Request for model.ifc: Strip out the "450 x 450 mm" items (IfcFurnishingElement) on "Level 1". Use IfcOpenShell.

First a look at what the model holds.

```python
import ifcopenshell
import ifcopenshell.util.element

model = ifcopenshell.open("model.ifc")
print(model.schema)
storey = next(s for s in model.by_type("IfcBuildingStorey") if s.Name == "Level 1")
furniture = [e for e in ifcopenshell.util.element.get_decomposition(storey) if e.is_a("IfcFurnishingElement")]
seen = {}
for e in furniture:
    element_type = ifcopenshell.util.element.get_type(e)
    name = element_type.Name if element_type not in (None, e) else None
    seen[name] = seen.get(name, 0) + 1
for name, count in sorted(seen.items(), key=str):
    print(count, "x", name)
```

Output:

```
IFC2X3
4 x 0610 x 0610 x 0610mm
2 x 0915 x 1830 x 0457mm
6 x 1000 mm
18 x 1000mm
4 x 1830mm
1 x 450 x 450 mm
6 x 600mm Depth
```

```python
import ifcopenshell
import ifcopenshell.api.root
import ifcopenshell.util.element

model = ifcopenshell.open("model.ifc")

storey = next(s for s in model.by_type("IfcBuildingStorey") if s.Name == "Level 1")
furniture = [e for e in ifcopenshell.util.element.get_decomposition(storey) if e.is_a("IfcFurnishingElement")]
targets = [e for e in furniture if (t := ifcopenshell.util.element.get_type(e)) not in (None, e) and t.Name == "450 x 450 mm"]

for e in targets:
    ifcopenshell.api.root.remove_product(model, product=e)
print(len(targets), "removed")

model.write("model-out.ifc")
```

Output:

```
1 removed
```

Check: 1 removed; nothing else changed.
